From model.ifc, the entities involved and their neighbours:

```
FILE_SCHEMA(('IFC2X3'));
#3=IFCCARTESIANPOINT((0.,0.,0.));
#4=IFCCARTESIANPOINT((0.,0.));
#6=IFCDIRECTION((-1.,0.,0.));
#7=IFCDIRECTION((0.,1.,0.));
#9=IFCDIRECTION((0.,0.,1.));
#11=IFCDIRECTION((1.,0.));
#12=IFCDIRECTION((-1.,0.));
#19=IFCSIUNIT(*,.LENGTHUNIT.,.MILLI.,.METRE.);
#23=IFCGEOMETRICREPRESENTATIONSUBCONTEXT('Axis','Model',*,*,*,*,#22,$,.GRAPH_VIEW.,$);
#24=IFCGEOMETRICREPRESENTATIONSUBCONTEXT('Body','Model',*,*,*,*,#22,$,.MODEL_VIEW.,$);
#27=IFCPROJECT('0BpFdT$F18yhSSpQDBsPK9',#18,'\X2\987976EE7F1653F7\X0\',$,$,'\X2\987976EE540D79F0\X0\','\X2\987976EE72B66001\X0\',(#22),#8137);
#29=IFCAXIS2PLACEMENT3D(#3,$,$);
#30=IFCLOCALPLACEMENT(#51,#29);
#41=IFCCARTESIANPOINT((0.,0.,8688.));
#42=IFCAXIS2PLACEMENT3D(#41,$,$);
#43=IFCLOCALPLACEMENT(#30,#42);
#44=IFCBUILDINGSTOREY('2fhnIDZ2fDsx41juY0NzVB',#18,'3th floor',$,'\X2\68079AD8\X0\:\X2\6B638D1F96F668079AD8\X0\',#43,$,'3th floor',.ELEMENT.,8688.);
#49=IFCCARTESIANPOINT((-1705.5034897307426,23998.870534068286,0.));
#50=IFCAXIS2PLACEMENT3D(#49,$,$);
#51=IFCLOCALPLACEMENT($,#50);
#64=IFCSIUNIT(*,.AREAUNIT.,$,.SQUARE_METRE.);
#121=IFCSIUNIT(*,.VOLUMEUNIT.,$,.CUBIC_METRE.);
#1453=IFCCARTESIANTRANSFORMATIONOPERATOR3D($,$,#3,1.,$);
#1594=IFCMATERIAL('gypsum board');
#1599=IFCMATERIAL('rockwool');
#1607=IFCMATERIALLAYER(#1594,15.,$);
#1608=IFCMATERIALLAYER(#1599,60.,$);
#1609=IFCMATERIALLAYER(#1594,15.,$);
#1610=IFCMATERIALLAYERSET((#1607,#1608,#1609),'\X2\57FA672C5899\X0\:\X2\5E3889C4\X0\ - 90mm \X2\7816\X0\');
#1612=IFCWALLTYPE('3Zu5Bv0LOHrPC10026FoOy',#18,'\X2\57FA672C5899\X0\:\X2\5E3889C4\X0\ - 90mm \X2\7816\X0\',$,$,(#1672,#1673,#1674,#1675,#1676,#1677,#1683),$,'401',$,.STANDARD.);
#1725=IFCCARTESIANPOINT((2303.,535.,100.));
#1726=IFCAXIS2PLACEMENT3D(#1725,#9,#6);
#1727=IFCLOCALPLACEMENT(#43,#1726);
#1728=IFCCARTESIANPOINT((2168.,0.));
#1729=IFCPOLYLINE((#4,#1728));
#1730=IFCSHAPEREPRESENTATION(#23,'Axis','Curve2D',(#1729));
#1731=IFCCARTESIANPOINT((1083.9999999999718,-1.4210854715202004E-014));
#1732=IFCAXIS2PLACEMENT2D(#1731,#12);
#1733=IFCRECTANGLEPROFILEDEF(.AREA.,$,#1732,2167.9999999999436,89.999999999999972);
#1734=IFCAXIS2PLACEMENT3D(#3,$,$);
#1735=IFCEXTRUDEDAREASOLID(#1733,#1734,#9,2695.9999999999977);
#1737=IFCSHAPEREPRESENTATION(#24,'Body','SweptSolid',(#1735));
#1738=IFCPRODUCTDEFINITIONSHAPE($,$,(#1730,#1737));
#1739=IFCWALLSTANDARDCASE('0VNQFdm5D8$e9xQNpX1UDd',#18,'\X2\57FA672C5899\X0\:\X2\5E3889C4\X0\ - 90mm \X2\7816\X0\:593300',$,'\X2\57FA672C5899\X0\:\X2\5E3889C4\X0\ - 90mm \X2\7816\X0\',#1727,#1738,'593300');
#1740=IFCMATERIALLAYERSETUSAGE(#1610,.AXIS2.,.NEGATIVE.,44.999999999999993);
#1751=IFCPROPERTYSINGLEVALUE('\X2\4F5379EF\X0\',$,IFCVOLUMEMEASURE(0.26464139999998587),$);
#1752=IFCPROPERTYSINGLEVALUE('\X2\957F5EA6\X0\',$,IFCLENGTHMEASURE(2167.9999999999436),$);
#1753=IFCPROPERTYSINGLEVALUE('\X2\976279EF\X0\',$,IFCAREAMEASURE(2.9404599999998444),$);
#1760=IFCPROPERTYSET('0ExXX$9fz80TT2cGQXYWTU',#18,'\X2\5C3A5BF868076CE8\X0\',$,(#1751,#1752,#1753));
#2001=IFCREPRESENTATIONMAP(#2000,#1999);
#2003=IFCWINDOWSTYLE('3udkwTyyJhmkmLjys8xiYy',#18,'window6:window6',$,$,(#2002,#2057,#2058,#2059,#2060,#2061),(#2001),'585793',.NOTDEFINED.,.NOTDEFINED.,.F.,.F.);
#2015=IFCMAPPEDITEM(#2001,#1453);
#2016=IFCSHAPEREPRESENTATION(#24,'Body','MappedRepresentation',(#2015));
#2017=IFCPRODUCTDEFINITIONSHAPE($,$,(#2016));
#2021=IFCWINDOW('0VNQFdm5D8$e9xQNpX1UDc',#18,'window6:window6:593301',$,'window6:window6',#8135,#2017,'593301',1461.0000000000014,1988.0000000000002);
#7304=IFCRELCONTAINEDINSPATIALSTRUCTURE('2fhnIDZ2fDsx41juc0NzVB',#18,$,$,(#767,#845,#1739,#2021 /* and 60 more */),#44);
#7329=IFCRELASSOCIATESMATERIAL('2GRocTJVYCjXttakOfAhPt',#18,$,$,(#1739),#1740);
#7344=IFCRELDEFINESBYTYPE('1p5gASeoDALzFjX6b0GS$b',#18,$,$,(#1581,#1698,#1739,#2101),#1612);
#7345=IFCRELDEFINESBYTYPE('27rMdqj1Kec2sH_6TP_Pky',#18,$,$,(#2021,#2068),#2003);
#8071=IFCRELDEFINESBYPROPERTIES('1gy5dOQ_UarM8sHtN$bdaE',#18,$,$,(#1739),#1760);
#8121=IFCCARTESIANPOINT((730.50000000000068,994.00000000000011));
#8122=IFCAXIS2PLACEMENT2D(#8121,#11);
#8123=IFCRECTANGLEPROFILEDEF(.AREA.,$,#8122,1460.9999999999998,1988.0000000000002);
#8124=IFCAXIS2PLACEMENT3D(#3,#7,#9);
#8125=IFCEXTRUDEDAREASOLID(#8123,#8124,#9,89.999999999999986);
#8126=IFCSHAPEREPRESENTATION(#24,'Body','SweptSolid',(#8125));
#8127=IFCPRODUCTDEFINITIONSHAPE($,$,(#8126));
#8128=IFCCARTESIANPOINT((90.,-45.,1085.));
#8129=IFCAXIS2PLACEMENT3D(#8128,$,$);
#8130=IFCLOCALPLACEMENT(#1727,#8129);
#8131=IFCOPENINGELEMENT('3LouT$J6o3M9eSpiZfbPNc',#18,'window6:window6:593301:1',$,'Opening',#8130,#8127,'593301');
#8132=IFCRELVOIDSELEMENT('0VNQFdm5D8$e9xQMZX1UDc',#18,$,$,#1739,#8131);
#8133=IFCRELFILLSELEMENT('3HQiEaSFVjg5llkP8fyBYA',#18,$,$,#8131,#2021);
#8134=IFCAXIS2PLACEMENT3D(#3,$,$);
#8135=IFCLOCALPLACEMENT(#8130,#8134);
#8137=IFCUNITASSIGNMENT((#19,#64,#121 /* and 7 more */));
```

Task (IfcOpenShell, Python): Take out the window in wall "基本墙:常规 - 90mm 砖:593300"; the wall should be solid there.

```python
import ifcopenshell
import ifcopenshell.api.feature
import ifcopenshell.api.pset
import ifcopenshell.api.root
import ifcopenshell.geom
import ifcopenshell.util.element
import ifcopenshell.util.shape
import ifcopenshell.util.unit

model = ifcopenshell.open("model.ifc")
area_scale = ifcopenshell.util.unit.calculate_unit_scale(model, "AREAUNIT")
volume_scale = ifcopenshell.util.unit.calculate_unit_scale(model, "VOLUMEUNIT")
settings = ifcopenshell.geom.settings()


def volume(element):
    """Net volume in cubic metres, openings subtracted."""
    shape = ifcopenshell.geom.create_shape(settings, element)
    return ifcopenshell.util.shape.get_volume(shape.geometry)


window = model.by_guid("0VNQFdm5D8$e9xQNpX1UDc")
opening = window.FillsVoids[0].RelatingOpeningElement
wall = opening.VoidsElements[0].RelatingBuildingElement
before = volume(wall)

ifcopenshell.api.root.remove_product(model, product=window)
ifcopenshell.api.feature.remove_feature(model, feature=opening)

after = volume(wall)
thickness = 0.09  # wall thickness in metres

# Update the wall's stored quantities.
pset = model.by_id(ifcopenshell.util.element.get_pset(wall, "尺寸标注", should_inherit=False)["id"])
ifcopenshell.api.pset.edit_pset(model, pset=pset, properties={
    "体积": model.create_entity("IfcVolumeMeasure", after / volume_scale),
    "面积": model.create_entity("IfcAreaMeasure", after / thickness / area_scale),
})

print(f"wall volume {before:.3f} -> {after:.3f} m3")

model.write("model-out.ifc")
```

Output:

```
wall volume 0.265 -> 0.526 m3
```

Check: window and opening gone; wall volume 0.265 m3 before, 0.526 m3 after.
